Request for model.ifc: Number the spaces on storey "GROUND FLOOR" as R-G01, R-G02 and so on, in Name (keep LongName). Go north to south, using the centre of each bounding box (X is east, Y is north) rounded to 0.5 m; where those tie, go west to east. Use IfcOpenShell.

First a look at what the model holds.

```python
import ifcopenshell
import ifcopenshell.util.element
import ifcopenshell.util.placement

model = ifcopenshell.open("model.ifc")
print(model.schema)
storey = next(s for s in model.by_type("IfcBuildingStorey") if s.Name == "GROUND FLOOR")
spaces = [e for e in ifcopenshell.util.element.get_decomposition(storey) if e.is_a("IfcSpace")]
for e in sorted(spaces, key=lambda e: e.id()):
    origin = ifcopenshell.util.placement.get_local_placement(e.ObjectPlacement)[:3, 3]
    print(e.id(), e.Name, e.LongName, origin.round(2) + 0.0, sep=" | ")
```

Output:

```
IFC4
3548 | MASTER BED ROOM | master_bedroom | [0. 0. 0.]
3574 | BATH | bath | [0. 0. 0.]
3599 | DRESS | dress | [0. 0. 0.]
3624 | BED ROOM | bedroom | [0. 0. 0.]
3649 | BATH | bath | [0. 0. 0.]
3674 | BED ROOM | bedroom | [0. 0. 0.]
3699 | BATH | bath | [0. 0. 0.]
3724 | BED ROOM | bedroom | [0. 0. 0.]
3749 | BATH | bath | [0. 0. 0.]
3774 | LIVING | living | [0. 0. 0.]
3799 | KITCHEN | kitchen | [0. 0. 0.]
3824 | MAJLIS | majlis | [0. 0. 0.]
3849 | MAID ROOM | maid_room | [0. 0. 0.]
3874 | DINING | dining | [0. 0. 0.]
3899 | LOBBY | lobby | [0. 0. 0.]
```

```python
import ifcopenshell
import ifcopenshell.geom
import ifcopenshell.util.element
import ifcopenshell.util.shape

model = ifcopenshell.open("model.ifc")
settings = ifcopenshell.geom.settings()
settings.set("use-world-coords", True)


def centre(element):
    shape = ifcopenshell.geom.create_shape(settings, element)
    return ifcopenshell.util.shape.get_bbox_centroid(shape.geometry)


storey = next(s for s in model.by_type("IfcBuildingStorey") if s.Name == "GROUND FLOOR")
spaces = [e for e in ifcopenshell.util.element.get_decomposition(storey) if e.is_a("IfcSpace")]

# Insertion points can sit at a corner or the storey origin, so sort by the geometry (in metres).
centres = {e: centre(e) for e in spaces}
spaces.sort(key=lambda e: (-round(centres[e][1] / 0.5), centres[e][0]))

for i, e in enumerate(spaces, start=1):
    number = f"R-G{i:02d}"
    e.Name = number
    print(e.id(), number)

model.write("model_v2.ifc")
```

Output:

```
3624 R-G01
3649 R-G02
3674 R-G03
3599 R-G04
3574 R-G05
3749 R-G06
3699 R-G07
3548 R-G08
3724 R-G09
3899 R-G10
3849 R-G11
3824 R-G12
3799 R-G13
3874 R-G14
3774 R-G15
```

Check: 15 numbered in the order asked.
